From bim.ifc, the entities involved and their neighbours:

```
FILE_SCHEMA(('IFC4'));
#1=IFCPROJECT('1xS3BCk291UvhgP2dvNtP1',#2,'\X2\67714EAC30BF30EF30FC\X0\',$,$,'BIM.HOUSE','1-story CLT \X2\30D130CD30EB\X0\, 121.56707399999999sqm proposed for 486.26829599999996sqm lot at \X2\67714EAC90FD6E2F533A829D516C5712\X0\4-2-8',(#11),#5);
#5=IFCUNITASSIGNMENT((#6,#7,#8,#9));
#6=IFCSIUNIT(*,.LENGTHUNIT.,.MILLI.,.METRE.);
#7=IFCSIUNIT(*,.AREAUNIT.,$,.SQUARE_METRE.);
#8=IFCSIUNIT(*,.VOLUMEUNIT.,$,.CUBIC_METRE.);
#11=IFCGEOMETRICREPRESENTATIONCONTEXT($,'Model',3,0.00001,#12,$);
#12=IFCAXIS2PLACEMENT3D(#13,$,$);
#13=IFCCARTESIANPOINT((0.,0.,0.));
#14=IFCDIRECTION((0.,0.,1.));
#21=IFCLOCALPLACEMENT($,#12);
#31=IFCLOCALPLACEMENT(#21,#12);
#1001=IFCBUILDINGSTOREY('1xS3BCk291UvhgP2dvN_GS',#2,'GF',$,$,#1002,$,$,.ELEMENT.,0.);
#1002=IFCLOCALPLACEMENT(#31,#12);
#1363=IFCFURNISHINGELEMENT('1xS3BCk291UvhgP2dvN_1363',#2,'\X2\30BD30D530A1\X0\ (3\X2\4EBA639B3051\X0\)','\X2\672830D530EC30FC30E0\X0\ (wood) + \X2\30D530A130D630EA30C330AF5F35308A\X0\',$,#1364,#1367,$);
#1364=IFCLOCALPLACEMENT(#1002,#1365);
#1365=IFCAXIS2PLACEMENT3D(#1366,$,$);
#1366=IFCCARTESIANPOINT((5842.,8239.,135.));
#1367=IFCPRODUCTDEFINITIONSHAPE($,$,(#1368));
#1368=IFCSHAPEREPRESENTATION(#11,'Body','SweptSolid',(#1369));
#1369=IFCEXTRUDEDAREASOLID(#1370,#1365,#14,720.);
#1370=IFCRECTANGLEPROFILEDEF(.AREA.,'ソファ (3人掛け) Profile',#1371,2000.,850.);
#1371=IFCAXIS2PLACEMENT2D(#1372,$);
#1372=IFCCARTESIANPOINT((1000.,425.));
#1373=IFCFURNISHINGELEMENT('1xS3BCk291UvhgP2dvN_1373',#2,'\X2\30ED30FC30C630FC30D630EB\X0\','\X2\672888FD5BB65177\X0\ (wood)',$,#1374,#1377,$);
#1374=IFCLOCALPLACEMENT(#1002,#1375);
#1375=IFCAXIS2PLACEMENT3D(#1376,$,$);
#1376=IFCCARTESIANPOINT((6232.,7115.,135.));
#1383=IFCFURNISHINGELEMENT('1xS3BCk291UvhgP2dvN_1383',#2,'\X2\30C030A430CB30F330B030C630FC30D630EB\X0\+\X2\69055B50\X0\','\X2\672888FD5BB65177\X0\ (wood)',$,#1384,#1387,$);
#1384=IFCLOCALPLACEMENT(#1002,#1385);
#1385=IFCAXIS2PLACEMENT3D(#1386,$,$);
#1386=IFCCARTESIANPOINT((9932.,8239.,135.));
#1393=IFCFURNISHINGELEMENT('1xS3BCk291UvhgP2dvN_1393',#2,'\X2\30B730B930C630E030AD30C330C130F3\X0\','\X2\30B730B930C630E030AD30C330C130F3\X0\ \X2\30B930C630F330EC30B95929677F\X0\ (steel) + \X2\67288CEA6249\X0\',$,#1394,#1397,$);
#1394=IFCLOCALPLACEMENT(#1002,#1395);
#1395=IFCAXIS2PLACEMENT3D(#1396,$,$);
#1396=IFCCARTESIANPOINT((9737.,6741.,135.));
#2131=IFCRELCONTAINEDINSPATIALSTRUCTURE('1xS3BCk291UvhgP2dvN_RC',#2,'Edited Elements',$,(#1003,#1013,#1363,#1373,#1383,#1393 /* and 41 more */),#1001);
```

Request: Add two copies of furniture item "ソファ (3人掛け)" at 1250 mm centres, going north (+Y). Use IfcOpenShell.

```python
import numpy as np
import ifcopenshell
import ifcopenshell.api.geometry
import ifcopenshell.api.root
import ifcopenshell.util.element
import ifcopenshell.util.placement

model = ifcopenshell.open("bim.ifc")


def reuse_history(source, copy):
    """copy_class also copies each property set's owner history, people and application; keep the originals."""
    for rel in copy.IsDefinedBy:
        if rel.is_a("IfcRelDefinesByProperties") and (history := rel.RelatingPropertyDefinition.OwnerHistory):
            rel.RelatingPropertyDefinition.OwnerHistory = source.OwnerHistory
            ifcopenshell.util.element.remove_deep2(model, history)


source = model.by_id(1363)
base = ifcopenshell.util.placement.get_local_placement(source.ObjectPlacement)
step = np.array([0.0, 1.0, 0.0]) * 1250.0

for i in range(1, 3):
    copy = ifcopenshell.api.root.copy_class(model, product=source)
    copy.Representation = ifcopenshell.util.element.copy_deep(
        model, source.Representation, exclude=["IfcGeometricRepresentationContext", "IfcRepresentationMap"]
    )
    reuse_history(source, copy)
    matrix = base.copy()
    matrix[:3, 3] += i * step
    print("added at", matrix[:3, 3].round(3) + 0.0)
    ifcopenshell.api.geometry.edit_object_placement(model, product=copy, matrix=matrix, is_si=False)

model.write("bim_rev.ifc")
```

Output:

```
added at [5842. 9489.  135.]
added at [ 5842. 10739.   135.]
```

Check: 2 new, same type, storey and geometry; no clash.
